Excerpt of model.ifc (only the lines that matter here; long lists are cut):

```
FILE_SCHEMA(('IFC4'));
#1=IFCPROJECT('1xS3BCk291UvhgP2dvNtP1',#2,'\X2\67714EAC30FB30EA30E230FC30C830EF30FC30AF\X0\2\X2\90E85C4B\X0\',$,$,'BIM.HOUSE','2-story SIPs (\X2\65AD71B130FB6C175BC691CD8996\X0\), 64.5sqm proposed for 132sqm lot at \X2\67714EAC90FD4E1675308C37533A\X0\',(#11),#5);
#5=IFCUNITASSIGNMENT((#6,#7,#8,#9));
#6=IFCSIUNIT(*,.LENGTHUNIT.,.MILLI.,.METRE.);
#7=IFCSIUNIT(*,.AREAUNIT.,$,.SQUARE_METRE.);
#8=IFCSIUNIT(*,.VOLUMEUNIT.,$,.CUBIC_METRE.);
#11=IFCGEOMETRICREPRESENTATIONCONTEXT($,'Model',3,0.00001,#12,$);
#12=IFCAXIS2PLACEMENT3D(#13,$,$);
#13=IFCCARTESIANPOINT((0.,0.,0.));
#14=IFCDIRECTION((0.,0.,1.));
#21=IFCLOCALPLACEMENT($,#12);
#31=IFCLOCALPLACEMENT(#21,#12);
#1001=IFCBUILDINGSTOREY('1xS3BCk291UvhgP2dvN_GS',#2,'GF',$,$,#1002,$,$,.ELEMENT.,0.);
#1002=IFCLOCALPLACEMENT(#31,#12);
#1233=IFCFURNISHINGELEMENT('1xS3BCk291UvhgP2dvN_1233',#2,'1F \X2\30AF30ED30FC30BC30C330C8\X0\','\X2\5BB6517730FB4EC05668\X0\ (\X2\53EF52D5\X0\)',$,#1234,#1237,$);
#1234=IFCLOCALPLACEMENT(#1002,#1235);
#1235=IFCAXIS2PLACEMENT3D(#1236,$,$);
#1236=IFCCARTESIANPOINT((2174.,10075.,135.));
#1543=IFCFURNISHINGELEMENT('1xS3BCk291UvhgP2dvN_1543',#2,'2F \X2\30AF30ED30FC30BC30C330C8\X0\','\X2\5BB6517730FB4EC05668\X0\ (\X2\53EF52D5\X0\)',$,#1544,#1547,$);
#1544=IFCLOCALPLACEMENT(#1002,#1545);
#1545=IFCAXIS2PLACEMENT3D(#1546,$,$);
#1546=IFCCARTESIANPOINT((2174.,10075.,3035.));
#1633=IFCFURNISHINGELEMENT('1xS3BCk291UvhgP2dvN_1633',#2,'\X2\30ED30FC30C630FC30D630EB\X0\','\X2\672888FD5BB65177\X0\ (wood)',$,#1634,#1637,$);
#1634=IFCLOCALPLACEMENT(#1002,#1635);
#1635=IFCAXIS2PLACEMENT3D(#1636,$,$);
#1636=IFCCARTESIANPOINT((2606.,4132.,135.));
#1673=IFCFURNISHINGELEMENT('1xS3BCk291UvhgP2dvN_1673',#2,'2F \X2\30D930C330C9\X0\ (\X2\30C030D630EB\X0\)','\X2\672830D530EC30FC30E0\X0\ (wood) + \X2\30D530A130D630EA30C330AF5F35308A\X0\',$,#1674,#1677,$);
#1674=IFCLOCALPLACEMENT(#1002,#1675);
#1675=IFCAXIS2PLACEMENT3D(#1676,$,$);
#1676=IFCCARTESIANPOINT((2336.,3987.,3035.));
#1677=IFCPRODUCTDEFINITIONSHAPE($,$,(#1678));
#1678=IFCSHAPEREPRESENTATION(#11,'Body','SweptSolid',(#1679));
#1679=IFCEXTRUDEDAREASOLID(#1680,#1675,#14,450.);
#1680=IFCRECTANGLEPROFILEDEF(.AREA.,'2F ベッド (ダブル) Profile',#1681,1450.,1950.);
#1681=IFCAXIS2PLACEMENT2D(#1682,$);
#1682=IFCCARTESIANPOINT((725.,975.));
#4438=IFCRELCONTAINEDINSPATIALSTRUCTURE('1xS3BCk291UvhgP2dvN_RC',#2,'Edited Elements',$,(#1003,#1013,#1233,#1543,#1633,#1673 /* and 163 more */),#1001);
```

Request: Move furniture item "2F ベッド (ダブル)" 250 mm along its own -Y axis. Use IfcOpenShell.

```python
import ifcopenshell
import ifcopenshell.api.geometry
import ifcopenshell.util.placement

model = ifcopenshell.open("model.ifc")

item = model.by_guid("1xS3BCk291UvhgP2dvN_1673")
matrix = ifcopenshell.util.placement.get_local_placement(item.ObjectPlacement)
matrix[:3, 3] -= matrix[:3, 1] * 250.0
ifcopenshell.api.geometry.edit_object_placement(model, product=item, matrix=matrix, is_si=False)

print(ifcopenshell.util.placement.get_local_placement(item.ObjectPlacement).round(3) + 0.0)

model.write("model_edited.ifc")
```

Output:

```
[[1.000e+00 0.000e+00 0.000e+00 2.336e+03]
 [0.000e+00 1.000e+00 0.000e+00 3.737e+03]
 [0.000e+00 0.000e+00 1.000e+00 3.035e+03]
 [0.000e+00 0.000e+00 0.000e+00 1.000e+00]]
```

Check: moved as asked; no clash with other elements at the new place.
